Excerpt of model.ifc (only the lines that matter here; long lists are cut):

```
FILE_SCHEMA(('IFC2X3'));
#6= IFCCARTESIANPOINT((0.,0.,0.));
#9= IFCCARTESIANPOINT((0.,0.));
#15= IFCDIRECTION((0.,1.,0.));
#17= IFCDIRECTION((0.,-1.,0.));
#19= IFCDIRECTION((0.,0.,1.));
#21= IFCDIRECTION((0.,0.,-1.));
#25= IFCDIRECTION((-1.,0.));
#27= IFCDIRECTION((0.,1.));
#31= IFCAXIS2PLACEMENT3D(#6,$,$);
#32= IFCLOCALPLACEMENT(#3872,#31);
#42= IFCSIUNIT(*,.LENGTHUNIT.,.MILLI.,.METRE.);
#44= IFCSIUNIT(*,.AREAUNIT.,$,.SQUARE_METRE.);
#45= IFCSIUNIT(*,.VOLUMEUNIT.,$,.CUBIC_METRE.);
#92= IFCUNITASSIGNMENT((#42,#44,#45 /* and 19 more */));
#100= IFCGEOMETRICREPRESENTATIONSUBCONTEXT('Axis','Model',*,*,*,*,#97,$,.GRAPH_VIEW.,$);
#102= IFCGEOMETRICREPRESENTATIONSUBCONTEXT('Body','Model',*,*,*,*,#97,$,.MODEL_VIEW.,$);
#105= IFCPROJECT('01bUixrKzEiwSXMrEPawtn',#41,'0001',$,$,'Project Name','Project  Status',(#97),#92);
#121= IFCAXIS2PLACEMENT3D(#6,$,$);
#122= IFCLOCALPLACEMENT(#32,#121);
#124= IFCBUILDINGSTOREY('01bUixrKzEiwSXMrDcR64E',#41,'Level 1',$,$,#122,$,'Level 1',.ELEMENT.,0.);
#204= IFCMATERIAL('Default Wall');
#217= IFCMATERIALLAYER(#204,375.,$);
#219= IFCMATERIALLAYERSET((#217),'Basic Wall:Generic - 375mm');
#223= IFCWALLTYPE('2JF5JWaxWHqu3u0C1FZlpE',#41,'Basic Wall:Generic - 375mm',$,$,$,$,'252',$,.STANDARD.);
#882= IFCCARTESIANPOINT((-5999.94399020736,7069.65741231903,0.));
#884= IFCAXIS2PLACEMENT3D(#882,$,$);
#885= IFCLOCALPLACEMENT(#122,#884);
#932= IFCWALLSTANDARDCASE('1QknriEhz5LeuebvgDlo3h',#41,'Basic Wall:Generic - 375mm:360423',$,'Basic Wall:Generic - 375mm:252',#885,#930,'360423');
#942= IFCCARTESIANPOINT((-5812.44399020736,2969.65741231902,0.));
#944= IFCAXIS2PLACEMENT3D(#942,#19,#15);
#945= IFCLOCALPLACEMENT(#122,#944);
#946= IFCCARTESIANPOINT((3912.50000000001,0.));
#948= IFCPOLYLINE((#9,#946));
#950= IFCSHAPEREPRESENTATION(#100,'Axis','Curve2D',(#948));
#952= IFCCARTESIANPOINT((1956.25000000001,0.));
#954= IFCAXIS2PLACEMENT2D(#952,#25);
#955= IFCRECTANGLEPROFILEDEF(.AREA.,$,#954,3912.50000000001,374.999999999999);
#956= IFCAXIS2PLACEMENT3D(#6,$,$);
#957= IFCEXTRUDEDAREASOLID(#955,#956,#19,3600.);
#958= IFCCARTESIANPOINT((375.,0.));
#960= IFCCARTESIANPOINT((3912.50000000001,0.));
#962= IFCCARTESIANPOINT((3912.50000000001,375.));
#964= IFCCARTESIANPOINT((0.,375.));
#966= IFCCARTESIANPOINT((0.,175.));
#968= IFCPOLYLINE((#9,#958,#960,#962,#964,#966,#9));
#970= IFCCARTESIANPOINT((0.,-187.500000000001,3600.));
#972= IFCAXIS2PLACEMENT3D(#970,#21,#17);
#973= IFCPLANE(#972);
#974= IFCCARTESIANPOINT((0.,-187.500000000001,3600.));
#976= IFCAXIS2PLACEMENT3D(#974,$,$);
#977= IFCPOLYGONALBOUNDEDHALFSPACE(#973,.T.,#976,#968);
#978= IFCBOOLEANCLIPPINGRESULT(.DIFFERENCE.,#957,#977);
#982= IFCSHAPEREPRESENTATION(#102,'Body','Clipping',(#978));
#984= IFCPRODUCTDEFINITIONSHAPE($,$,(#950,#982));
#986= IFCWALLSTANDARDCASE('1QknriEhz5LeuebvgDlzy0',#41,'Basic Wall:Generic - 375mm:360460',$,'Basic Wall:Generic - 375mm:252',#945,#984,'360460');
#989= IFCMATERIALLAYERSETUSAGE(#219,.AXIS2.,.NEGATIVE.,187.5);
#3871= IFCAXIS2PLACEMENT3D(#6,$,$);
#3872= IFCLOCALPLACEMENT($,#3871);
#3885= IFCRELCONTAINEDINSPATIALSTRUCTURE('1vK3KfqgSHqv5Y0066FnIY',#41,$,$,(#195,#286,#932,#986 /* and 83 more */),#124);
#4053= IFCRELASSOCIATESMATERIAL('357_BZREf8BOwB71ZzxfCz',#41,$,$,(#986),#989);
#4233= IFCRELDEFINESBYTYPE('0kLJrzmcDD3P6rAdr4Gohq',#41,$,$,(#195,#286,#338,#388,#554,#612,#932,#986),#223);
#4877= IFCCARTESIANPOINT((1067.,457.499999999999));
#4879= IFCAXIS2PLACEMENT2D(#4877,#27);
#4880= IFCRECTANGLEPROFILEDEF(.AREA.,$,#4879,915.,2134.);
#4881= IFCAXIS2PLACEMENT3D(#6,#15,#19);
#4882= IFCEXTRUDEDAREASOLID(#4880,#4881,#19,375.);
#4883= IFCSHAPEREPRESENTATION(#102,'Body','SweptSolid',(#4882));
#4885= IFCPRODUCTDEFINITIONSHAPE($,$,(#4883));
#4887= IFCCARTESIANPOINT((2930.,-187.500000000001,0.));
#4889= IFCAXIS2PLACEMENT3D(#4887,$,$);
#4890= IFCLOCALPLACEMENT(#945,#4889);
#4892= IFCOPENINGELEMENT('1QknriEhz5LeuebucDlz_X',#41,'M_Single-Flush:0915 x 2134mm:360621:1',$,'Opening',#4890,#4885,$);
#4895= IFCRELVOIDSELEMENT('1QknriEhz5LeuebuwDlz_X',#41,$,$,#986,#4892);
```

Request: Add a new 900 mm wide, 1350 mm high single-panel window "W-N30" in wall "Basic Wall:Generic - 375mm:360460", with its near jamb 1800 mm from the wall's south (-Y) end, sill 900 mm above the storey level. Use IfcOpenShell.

```python
import numpy as np
import ifcopenshell
import ifcopenshell.api.feature
import ifcopenshell.api.geometry
import ifcopenshell.api.root
import ifcopenshell.api.spatial
import ifcopenshell.api.type
import ifcopenshell.geom
import ifcopenshell.util.element
import ifcopenshell.util.placement
import ifcopenshell.util.representation
import ifcopenshell.util.shape
import ifcopenshell.util.unit

model = ifcopenshell.open("model.ifc")
unit_scale = ifcopenshell.util.unit.calculate_unit_scale(model)
settings = ifcopenshell.geom.settings()


def volume(element):
    """Net volume in cubic metres, openings subtracted."""
    shape = ifcopenshell.geom.create_shape(settings, element)
    return ifcopenshell.util.shape.get_volume(shape.geometry)


wall = model.by_guid("1QknriEhz5LeuebvgDlzy0")
storey = ifcopenshell.util.element.get_container(wall, ifc_class="IfcBuildingStorey")
context = ifcopenshell.util.representation.get_context(model, "Model", "Body", "MODEL_VIEW")
before = volume(wall)

width, height, from_end, sill = 0.9, 1.35, 1.8, 0.9  # metres

# The wall runs along its own X axis, and the end named is its -X end.
wall_shape = ifcopenshell.geom.create_shape(settings, wall)
x, y, z = ifcopenshell.util.shape.get_vertices(wall_shape.geometry).T
start = x.min() + from_end
face, thickness = float(y.min()), float(y.max() - y.min())
wall_matrix = ifcopenshell.util.placement.get_local_placement(wall.ObjectPlacement)
level = ifcopenshell.util.placement.get_local_placement(storey.ObjectPlacement)[2, 3]


def in_wall(x, y):
    """Placement at x, y metres in the wall's axes, at sill height."""
    matrix = wall_matrix.copy()
    matrix[:, 3] = wall_matrix @ np.array([x / unit_scale, y / unit_scale, 0.0, 1.0])
    matrix[2, 3] = level + sill / unit_scale
    return matrix


# Opening: a box that overshoots both wall faces by 50 mm.
opening = ifcopenshell.api.root.create_entity(model, ifc_class="IfcOpeningElement")
box = ifcopenshell.api.geometry.add_wall_representation(
    model, context=context, length=width, height=height, thickness=thickness + 0.1
)
ifcopenshell.api.geometry.assign_representation(model, product=opening, representation=box)
ifcopenshell.api.geometry.edit_object_placement(model, product=opening, matrix=in_wall(start, face - 0.05), is_si=False)
ifcopenshell.api.feature.add_feature(model, feature=opening, element=wall)

window = ifcopenshell.api.root.create_entity(model, ifc_class="IfcWindow", name="W-N30")
window.OverallWidth, window.OverallHeight = width / unit_scale, height / unit_scale
body = ifcopenshell.api.geometry.add_window_representation(
    model,
    context=context,
    overall_width=window.OverallWidth,
    overall_height=window.OverallHeight,
    partition_type="SINGLE_PANEL",
)
ifcopenshell.api.geometry.assign_representation(model, product=window, representation=body)
ifcopenshell.api.spatial.assign_container(model, products=[window], relating_structure=storey)
fills = ifcopenshell.api.feature.add_filling(model, opening=opening, element=window)
fills.OwnerHistory = window.OwnerHistory  # required in IFC2X3

# IFC2X3 keeps the operation on the window style.
style = ifcopenshell.api.root.create_entity(model, ifc_class="IfcWindowStyle", name="W-N30")
style.OperationType, style.ConstructionType = "SINGLE_PANEL", "NOTDEFINED"
style.ParameterTakesPrecedence = style.Sizeable = False
ifcopenshell.api.type.assign_type(model, related_objects=[window], relating_type=style)

# Centre the window in the wall's thickness.
ifcopenshell.api.geometry.edit_object_placement(model, product=window, matrix=in_wall(start, face), is_si=False)
window_shape = ifcopenshell.geom.create_shape(settings, window)
depth = ifcopenshell.util.shape.get_vertices(window_shape.geometry)[:, 1]
offset = face + thickness / 2 - (depth.min() + depth.max()) / 2
ifcopenshell.api.geometry.edit_object_placement(model, product=window, matrix=in_wall(start, offset), is_si=False)

after = volume(wall)

print(f"wall volume {before:.3f} -> {after:.3f} m3")

model.write("model_rev.ifc")
```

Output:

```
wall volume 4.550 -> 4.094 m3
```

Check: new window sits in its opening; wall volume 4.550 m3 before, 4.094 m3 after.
